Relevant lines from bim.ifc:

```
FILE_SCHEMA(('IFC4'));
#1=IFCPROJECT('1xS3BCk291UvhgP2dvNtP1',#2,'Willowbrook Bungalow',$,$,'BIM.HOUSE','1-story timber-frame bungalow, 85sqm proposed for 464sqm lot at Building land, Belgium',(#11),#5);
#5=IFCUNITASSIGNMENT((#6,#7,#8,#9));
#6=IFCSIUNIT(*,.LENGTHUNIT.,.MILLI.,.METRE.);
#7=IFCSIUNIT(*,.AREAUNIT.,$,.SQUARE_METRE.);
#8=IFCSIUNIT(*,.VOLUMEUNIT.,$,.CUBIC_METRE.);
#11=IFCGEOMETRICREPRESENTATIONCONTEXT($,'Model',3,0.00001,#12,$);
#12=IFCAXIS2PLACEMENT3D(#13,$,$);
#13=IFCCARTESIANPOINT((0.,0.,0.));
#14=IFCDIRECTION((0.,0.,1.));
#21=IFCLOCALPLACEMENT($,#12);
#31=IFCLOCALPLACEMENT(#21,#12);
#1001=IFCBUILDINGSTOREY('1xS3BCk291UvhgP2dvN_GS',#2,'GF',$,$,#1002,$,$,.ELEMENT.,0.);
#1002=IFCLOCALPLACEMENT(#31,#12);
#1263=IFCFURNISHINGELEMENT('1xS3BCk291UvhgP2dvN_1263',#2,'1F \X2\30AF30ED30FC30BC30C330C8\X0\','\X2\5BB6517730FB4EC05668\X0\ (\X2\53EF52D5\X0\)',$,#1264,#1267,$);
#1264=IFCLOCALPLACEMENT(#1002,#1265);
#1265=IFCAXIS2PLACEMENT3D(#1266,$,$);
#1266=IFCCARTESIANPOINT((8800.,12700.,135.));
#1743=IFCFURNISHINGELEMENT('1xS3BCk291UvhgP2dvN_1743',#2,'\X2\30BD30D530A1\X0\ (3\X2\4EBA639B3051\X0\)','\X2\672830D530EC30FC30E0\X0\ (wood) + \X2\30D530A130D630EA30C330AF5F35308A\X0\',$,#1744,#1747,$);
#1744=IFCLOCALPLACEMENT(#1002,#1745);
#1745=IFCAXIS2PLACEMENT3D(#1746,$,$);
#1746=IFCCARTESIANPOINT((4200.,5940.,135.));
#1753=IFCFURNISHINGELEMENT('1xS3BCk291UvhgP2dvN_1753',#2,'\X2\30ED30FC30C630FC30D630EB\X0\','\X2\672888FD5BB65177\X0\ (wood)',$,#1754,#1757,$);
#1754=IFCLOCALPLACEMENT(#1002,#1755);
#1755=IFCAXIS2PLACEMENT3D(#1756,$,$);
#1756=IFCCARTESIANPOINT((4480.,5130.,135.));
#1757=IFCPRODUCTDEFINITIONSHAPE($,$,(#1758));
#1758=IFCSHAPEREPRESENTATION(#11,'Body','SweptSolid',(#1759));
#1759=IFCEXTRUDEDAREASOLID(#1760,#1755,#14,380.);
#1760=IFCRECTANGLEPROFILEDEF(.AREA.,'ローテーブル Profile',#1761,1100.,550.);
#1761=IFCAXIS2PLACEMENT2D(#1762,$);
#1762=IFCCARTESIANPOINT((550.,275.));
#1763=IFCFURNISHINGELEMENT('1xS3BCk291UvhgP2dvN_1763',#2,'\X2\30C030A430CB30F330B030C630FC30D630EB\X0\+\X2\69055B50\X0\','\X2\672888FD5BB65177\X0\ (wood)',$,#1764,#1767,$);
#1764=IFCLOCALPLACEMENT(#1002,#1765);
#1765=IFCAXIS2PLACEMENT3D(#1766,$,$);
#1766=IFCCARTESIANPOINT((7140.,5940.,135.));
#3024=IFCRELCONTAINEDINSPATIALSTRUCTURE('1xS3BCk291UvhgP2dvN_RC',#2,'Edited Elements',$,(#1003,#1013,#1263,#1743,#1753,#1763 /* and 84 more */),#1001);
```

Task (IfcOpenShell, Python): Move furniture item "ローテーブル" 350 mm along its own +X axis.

```python
import ifcopenshell
import ifcopenshell.api.geometry
import ifcopenshell.util.placement
import ifcopenshell.util.unit

model = ifcopenshell.open("bim.ifc")
unit_scale = ifcopenshell.util.unit.calculate_unit_scale(model)

item = model.by_guid("1xS3BCk291UvhgP2dvN_1753")
matrix = ifcopenshell.util.placement.get_local_placement(item.ObjectPlacement)
matrix[:3, 3] += matrix[:3, 0] * 0.35 / unit_scale
ifcopenshell.api.geometry.edit_object_placement(model, product=item, matrix=matrix, is_si=False)

print(ifcopenshell.util.placement.get_local_placement(item.ObjectPlacement).round(3) + 0.0)

model.write("bim_edited.ifc")
```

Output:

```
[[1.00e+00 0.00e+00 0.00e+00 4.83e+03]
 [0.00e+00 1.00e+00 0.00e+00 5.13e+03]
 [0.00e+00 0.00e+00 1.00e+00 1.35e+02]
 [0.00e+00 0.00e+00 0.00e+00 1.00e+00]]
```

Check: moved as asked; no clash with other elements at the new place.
